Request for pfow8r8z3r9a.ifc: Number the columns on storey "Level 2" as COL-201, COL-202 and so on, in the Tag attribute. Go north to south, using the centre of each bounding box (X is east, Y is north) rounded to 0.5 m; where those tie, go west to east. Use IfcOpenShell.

First a look at what the model holds.

```python
import ifcopenshell
import ifcopenshell.util.element
import ifcopenshell.util.placement

model = ifcopenshell.open("pfow8r8z3r9a.ifc")
print(model.schema)
storey = next(s for s in model.by_type("IfcBuildingStorey") if s.Name == "Level 2")
columns = [e for e in ifcopenshell.util.element.get_decomposition(storey) if e.is_a("IfcColumn")]
for e in sorted(columns, key=lambda e: e.id()):
    origin = ifcopenshell.util.placement.get_local_placement(e.ObjectPlacement)[:3, 3]
    print(e.id(), e.Tag, e.Name, origin.round(2) + 0.0, sep=" | ")
```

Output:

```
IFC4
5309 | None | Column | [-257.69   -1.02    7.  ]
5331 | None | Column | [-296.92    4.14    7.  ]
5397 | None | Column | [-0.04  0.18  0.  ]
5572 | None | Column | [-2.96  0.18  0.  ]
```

```python
import ifcopenshell
import ifcopenshell.geom
import ifcopenshell.util.element
import ifcopenshell.util.shape

model = ifcopenshell.open("pfow8r8z3r9a.ifc")
settings = ifcopenshell.geom.settings()
settings.set("use-world-coords", True)


def centre(element):
    shape = ifcopenshell.geom.create_shape(settings, element)
    return ifcopenshell.util.shape.get_bbox_centroid(shape.geometry)


storey = next(s for s in model.by_type("IfcBuildingStorey") if s.Name == "Level 2")
columns = [e for e in ifcopenshell.util.element.get_decomposition(storey) if e.is_a("IfcColumn")]

# Insertion points can sit at a corner or the storey origin, so sort by the geometry (in metres).
centres = {e: centre(e) for e in columns}
columns.sort(key=lambda e: (-round(centres[e][1] / 0.5), centres[e][0]))

for i, e in enumerate(columns, start=1):
    number = f"COL-2{i:02d}"
    e.Tag = number
    print(e.id(), number)

model.write("pfow8r8z3r9a_edited.ifc")
```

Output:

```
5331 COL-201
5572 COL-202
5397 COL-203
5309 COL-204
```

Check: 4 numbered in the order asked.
